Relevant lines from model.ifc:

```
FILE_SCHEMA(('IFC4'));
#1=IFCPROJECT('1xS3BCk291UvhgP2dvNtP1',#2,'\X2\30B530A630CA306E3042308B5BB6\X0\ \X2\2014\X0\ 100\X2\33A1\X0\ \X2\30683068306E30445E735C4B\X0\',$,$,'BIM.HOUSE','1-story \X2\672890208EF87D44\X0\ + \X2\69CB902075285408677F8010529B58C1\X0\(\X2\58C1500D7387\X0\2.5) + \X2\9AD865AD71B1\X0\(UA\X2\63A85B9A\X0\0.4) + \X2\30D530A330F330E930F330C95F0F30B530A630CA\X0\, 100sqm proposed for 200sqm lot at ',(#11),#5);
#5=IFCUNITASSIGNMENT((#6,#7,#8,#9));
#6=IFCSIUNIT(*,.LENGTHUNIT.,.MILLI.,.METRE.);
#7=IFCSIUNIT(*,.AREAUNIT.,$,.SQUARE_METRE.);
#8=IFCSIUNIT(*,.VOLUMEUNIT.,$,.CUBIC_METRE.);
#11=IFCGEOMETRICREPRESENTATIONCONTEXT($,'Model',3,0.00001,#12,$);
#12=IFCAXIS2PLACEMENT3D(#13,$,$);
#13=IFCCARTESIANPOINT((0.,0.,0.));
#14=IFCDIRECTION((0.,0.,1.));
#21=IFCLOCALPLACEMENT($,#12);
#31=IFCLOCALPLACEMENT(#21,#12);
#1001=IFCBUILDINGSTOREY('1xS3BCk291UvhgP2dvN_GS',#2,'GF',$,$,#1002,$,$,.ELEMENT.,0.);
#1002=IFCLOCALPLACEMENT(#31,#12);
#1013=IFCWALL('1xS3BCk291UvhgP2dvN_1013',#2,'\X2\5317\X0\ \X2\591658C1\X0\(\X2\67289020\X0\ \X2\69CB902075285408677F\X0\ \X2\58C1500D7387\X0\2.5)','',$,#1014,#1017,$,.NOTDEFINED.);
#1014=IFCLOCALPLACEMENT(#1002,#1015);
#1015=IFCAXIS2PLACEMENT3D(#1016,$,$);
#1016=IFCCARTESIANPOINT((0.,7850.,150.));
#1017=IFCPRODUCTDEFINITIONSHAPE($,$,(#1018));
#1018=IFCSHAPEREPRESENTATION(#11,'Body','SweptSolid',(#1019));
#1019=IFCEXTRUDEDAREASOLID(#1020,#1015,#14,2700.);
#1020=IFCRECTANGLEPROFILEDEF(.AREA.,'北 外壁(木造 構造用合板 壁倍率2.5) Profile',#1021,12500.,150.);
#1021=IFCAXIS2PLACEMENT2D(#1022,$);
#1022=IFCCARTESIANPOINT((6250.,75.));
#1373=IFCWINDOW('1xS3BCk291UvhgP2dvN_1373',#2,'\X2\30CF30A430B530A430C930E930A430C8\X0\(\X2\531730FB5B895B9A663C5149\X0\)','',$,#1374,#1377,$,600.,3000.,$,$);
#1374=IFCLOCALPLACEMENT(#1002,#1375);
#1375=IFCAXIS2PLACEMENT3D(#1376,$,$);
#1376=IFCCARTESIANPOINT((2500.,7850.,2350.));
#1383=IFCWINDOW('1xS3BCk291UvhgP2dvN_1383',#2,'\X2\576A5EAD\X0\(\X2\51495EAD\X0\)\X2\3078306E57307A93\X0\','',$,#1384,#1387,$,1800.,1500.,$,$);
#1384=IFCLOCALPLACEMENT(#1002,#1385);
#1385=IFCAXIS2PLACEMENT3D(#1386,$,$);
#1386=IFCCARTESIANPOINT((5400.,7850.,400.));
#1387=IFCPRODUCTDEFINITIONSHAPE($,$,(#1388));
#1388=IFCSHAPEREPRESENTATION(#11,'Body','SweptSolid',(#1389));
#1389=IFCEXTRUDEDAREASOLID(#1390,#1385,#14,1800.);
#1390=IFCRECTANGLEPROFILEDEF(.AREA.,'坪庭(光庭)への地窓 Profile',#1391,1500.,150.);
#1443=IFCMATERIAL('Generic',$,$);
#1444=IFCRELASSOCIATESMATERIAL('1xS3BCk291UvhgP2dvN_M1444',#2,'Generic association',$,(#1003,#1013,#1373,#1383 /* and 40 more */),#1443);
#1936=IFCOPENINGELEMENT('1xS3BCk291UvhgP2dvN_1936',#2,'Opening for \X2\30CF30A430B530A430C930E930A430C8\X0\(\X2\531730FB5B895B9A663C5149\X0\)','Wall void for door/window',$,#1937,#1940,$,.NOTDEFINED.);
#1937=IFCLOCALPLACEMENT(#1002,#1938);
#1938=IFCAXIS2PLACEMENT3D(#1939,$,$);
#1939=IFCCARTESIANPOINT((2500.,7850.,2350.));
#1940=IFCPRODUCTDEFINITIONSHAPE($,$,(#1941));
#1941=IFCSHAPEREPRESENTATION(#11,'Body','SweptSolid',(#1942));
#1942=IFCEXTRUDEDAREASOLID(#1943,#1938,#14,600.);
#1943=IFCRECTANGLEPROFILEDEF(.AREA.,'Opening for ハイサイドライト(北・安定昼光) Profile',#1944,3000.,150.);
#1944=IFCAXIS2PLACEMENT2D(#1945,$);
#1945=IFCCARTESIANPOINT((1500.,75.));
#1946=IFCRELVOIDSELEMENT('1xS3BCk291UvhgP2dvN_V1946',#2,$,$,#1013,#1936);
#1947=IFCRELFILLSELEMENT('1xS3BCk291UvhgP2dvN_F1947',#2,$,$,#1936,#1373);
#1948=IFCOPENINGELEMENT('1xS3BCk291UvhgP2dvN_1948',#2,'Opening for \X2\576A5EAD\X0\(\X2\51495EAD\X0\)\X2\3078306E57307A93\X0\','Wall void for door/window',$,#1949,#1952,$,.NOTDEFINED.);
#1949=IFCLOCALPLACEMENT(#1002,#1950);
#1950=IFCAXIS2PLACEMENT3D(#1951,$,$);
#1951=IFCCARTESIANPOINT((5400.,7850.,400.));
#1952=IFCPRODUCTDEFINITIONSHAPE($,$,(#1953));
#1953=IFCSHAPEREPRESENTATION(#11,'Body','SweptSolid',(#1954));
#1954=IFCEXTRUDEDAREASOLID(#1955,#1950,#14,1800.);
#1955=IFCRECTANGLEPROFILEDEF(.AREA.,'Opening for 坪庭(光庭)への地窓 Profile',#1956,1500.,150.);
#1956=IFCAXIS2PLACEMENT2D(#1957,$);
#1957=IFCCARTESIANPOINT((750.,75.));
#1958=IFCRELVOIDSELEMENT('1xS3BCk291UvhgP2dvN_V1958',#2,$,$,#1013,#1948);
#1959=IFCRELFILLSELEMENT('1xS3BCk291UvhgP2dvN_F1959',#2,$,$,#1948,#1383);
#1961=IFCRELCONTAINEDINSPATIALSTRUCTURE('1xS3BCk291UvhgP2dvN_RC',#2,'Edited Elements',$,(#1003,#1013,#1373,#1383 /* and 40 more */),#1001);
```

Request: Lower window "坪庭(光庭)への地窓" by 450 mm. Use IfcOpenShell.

```python
import numpy as np
import ifcopenshell
import ifcopenshell.api.geometry
import ifcopenshell.util.placement
import ifcopenshell.util.unit

model = ifcopenshell.open("model.ifc")
unit_scale = ifcopenshell.util.unit.calculate_unit_scale(model)

window = model.by_id(1383)
opening = window.FillsVoids[0].RelatingOpeningElement
dz = -0.45 / unit_scale

shift = np.array([0.0, 0.0, dz])
# The window is not placed relative to its opening, so move both.
for product in (opening, window):
    matrix = ifcopenshell.util.placement.get_local_placement(product.ObjectPlacement)
    matrix[:3, 3] += shift
    ifcopenshell.api.geometry.edit_object_placement(model, product=product, matrix=matrix, is_si=False)

print(f"moved by {dz * unit_scale:+.3f} m")

model.write("model_edited.ifc")
```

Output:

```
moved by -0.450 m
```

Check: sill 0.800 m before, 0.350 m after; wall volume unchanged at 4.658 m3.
